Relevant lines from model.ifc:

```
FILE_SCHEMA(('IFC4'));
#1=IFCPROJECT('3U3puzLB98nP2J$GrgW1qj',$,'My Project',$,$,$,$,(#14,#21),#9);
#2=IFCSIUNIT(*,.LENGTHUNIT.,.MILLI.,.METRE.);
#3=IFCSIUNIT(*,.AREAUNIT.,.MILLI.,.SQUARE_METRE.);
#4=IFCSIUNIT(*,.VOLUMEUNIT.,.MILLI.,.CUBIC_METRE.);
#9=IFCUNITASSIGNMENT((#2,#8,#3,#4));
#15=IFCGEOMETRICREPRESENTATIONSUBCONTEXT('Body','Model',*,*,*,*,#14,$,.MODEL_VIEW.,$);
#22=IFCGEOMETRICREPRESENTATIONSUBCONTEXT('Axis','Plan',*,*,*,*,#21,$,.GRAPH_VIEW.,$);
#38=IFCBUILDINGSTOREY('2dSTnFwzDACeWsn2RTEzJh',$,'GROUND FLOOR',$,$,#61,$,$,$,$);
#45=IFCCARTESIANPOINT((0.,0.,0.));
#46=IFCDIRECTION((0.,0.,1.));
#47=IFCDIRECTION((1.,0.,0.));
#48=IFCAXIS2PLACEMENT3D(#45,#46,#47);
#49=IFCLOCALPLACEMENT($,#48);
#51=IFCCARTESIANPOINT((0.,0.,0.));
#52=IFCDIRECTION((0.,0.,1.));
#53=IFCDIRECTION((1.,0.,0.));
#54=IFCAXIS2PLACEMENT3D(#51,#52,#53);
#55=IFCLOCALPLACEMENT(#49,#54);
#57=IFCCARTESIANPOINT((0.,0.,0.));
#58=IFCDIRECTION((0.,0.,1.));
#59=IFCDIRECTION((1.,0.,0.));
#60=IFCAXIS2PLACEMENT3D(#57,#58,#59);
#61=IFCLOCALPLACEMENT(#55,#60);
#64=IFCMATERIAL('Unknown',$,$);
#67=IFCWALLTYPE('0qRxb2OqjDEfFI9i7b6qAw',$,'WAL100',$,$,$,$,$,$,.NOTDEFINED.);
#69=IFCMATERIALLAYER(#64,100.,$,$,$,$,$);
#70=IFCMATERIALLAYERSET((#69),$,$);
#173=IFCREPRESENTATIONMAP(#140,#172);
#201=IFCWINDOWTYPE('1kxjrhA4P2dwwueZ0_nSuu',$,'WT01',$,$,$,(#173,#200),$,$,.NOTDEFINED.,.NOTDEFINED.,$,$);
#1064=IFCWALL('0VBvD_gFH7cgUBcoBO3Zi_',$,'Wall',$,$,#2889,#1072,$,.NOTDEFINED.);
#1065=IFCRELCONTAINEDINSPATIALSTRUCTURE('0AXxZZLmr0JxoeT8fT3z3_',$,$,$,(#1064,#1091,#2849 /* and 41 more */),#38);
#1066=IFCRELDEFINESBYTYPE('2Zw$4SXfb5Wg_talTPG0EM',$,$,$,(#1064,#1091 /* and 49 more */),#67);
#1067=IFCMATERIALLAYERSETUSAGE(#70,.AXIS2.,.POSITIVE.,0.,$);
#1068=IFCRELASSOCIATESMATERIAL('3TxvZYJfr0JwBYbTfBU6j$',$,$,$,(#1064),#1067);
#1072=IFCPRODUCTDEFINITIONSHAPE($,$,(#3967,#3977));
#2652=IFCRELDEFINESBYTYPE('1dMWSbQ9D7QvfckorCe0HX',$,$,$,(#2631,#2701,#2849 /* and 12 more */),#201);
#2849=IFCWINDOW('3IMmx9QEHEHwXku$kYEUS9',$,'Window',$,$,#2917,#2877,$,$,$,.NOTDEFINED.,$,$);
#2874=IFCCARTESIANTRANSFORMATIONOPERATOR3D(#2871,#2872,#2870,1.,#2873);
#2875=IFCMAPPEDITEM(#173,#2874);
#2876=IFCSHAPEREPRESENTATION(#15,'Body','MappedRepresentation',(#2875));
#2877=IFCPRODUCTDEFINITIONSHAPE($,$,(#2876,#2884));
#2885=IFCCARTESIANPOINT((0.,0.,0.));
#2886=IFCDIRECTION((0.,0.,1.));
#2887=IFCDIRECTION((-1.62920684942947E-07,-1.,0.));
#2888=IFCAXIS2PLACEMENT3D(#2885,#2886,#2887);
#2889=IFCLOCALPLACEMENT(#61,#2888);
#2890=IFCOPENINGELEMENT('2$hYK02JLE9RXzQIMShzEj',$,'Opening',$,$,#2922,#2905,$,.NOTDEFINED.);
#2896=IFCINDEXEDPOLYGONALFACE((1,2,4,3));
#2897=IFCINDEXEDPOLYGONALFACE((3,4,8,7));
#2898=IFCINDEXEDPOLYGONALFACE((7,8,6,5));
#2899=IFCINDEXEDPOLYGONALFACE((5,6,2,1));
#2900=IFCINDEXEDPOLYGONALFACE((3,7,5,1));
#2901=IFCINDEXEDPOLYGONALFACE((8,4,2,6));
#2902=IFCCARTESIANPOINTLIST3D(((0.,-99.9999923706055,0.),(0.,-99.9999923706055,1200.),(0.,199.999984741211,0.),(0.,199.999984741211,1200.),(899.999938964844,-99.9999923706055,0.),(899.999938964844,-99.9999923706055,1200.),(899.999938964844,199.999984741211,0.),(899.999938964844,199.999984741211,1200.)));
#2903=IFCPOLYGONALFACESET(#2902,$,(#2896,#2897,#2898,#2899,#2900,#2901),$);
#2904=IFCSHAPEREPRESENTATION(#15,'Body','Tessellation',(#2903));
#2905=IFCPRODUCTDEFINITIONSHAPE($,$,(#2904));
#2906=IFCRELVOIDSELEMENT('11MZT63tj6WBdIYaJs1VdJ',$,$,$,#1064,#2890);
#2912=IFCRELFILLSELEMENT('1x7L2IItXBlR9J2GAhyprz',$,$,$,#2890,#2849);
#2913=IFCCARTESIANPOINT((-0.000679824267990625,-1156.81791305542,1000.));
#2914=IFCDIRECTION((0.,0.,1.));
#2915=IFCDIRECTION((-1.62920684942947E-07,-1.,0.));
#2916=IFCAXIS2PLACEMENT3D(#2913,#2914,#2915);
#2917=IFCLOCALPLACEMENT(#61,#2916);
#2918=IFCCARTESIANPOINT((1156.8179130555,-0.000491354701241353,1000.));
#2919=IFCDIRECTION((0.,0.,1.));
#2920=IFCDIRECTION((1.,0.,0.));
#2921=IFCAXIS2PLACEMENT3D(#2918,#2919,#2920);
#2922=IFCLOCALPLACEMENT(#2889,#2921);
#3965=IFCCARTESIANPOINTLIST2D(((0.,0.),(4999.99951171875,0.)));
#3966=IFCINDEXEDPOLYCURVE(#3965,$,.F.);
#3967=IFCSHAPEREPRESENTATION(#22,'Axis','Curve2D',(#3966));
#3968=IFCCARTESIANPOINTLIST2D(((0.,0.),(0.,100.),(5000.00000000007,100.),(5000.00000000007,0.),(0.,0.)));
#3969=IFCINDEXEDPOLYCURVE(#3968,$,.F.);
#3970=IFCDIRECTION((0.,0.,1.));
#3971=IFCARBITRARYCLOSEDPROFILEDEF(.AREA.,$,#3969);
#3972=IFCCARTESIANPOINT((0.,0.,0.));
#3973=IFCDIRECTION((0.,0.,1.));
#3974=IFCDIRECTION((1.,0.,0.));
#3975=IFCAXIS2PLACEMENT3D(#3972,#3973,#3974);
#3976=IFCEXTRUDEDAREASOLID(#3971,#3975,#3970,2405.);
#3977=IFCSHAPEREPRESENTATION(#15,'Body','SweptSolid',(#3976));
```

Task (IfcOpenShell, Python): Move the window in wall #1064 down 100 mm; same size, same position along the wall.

```python
import numpy as np
import ifcopenshell
import ifcopenshell.api.geometry
import ifcopenshell.util.placement
import ifcopenshell.util.unit

model = ifcopenshell.open("model.ifc")
unit_scale = ifcopenshell.util.unit.calculate_unit_scale(model)

window = model.by_guid("3IMmx9QEHEHwXku$kYEUS9")
opening = window.FillsVoids[0].RelatingOpeningElement
dz = -100.0

shift = np.array([0.0, 0.0, dz])
# The window is not placed relative to its opening, so move both.
for product in (opening, window):
    matrix = ifcopenshell.util.placement.get_local_placement(product.ObjectPlacement)
    matrix[:3, 3] += shift
    ifcopenshell.api.geometry.edit_object_placement(model, product=product, matrix=matrix, is_si=False)

print(f"moved by {dz * unit_scale:+.3f} m")

model.write("model_v2.ifc")
```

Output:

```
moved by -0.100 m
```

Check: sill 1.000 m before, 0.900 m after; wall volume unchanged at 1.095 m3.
